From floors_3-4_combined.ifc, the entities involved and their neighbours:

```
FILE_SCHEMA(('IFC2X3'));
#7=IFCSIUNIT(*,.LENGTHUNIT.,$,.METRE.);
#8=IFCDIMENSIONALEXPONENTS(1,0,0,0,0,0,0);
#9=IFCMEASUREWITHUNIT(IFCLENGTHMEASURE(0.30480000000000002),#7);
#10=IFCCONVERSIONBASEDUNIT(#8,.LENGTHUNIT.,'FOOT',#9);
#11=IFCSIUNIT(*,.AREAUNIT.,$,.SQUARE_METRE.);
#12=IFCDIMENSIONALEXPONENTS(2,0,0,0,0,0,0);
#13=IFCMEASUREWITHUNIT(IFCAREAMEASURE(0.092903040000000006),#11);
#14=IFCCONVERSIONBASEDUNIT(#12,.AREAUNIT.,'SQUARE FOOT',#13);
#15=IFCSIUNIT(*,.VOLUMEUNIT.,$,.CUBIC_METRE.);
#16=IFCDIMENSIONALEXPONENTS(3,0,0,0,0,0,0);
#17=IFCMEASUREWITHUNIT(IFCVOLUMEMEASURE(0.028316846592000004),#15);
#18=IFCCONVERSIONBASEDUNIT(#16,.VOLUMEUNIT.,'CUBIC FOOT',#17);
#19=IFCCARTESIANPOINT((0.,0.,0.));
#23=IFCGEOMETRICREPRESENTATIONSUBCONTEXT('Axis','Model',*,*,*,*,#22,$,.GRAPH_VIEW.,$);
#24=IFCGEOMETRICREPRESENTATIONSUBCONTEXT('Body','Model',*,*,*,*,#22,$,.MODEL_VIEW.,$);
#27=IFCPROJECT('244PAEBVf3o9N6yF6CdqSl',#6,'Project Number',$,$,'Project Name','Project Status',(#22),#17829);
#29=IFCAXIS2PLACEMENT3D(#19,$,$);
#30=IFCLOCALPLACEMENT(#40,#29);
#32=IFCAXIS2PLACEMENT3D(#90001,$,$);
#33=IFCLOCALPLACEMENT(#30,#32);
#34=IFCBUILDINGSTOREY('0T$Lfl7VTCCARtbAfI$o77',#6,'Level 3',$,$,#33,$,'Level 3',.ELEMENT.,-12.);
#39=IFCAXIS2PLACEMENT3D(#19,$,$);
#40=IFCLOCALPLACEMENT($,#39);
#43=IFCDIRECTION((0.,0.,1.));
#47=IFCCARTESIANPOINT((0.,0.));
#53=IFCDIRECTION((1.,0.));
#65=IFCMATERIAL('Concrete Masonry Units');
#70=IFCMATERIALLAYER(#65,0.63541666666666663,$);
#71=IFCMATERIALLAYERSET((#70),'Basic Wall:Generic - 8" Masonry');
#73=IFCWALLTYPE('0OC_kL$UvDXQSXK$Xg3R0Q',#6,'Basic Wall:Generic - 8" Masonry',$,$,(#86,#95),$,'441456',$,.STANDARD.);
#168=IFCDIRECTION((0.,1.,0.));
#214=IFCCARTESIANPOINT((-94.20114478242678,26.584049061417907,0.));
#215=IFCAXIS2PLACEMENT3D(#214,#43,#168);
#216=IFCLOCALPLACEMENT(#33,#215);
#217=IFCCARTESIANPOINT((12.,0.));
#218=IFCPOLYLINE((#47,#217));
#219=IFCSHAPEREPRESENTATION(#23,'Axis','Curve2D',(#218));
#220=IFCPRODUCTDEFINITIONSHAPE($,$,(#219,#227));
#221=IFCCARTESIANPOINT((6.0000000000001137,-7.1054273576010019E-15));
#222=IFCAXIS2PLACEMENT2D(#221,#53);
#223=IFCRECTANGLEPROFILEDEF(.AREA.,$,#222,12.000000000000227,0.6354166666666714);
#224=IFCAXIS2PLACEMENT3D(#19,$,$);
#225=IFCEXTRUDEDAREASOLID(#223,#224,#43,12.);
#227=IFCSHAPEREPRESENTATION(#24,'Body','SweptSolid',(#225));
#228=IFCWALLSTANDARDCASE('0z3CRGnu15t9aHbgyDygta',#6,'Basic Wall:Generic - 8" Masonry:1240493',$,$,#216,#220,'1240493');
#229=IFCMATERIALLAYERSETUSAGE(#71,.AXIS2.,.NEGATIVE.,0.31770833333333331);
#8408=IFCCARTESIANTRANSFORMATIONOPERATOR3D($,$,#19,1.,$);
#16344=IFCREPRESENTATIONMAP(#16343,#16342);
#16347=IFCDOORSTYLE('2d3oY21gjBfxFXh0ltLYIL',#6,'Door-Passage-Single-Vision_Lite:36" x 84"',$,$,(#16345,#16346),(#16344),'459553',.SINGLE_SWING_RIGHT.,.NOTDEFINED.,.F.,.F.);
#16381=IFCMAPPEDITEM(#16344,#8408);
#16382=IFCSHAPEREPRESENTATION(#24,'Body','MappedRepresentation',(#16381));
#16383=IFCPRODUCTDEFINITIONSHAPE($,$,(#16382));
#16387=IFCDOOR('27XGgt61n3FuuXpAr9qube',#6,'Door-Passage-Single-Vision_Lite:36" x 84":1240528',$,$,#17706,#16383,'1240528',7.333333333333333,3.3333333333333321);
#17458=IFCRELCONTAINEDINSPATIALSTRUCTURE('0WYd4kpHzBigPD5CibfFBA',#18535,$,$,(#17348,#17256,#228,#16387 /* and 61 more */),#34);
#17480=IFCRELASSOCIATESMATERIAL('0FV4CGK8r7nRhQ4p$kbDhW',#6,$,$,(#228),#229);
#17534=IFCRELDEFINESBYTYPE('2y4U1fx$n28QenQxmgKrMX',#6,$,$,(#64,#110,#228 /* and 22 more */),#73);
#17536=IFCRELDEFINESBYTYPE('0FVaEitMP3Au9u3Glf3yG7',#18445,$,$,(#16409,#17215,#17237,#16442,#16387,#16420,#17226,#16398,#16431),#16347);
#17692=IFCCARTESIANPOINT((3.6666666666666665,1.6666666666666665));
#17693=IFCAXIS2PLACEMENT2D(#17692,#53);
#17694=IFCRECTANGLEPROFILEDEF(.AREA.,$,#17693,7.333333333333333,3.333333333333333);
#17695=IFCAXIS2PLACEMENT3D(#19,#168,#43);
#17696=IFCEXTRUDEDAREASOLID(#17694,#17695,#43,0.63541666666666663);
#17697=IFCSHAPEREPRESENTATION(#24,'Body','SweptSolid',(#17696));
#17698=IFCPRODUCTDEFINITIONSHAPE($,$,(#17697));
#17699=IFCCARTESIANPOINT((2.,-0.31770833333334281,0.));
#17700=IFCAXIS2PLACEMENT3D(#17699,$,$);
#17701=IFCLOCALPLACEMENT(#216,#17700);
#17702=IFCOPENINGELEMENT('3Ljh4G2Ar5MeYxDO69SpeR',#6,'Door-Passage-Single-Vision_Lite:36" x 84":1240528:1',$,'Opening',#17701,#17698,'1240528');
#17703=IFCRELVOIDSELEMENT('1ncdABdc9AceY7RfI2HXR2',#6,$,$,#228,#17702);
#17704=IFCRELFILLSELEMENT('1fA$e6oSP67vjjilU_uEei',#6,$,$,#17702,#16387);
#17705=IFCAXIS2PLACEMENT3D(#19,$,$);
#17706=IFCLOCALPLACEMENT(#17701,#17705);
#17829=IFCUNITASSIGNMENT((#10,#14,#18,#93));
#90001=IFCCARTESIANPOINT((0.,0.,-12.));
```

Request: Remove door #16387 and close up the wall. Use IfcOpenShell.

```python
import ifcopenshell
import ifcopenshell.api.feature
import ifcopenshell.api.root
import ifcopenshell.geom
import ifcopenshell.util.shape

model = ifcopenshell.open("floors_3-4_combined.ifc")
settings = ifcopenshell.geom.settings()


def volume(element):
    """Net volume in cubic metres, openings subtracted."""
    shape = ifcopenshell.geom.create_shape(settings, element)
    return ifcopenshell.util.shape.get_volume(shape.geometry)


door = model.by_guid("27XGgt61n3FuuXpAr9qube")
opening = door.FillsVoids[0].RelatingOpeningElement
wall = opening.VoidsElements[0].RelatingBuildingElement
before = volume(wall)

ifcopenshell.api.root.remove_product(model, product=door)
ifcopenshell.api.feature.remove_feature(model, feature=opening)

after = volume(wall)

print(f"wall volume {before:.3f} -> {after:.3f} m3")

model.write("floors_3-4_combined-out.ifc")
```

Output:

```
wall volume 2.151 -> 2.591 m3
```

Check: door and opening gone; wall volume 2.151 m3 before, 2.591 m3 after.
